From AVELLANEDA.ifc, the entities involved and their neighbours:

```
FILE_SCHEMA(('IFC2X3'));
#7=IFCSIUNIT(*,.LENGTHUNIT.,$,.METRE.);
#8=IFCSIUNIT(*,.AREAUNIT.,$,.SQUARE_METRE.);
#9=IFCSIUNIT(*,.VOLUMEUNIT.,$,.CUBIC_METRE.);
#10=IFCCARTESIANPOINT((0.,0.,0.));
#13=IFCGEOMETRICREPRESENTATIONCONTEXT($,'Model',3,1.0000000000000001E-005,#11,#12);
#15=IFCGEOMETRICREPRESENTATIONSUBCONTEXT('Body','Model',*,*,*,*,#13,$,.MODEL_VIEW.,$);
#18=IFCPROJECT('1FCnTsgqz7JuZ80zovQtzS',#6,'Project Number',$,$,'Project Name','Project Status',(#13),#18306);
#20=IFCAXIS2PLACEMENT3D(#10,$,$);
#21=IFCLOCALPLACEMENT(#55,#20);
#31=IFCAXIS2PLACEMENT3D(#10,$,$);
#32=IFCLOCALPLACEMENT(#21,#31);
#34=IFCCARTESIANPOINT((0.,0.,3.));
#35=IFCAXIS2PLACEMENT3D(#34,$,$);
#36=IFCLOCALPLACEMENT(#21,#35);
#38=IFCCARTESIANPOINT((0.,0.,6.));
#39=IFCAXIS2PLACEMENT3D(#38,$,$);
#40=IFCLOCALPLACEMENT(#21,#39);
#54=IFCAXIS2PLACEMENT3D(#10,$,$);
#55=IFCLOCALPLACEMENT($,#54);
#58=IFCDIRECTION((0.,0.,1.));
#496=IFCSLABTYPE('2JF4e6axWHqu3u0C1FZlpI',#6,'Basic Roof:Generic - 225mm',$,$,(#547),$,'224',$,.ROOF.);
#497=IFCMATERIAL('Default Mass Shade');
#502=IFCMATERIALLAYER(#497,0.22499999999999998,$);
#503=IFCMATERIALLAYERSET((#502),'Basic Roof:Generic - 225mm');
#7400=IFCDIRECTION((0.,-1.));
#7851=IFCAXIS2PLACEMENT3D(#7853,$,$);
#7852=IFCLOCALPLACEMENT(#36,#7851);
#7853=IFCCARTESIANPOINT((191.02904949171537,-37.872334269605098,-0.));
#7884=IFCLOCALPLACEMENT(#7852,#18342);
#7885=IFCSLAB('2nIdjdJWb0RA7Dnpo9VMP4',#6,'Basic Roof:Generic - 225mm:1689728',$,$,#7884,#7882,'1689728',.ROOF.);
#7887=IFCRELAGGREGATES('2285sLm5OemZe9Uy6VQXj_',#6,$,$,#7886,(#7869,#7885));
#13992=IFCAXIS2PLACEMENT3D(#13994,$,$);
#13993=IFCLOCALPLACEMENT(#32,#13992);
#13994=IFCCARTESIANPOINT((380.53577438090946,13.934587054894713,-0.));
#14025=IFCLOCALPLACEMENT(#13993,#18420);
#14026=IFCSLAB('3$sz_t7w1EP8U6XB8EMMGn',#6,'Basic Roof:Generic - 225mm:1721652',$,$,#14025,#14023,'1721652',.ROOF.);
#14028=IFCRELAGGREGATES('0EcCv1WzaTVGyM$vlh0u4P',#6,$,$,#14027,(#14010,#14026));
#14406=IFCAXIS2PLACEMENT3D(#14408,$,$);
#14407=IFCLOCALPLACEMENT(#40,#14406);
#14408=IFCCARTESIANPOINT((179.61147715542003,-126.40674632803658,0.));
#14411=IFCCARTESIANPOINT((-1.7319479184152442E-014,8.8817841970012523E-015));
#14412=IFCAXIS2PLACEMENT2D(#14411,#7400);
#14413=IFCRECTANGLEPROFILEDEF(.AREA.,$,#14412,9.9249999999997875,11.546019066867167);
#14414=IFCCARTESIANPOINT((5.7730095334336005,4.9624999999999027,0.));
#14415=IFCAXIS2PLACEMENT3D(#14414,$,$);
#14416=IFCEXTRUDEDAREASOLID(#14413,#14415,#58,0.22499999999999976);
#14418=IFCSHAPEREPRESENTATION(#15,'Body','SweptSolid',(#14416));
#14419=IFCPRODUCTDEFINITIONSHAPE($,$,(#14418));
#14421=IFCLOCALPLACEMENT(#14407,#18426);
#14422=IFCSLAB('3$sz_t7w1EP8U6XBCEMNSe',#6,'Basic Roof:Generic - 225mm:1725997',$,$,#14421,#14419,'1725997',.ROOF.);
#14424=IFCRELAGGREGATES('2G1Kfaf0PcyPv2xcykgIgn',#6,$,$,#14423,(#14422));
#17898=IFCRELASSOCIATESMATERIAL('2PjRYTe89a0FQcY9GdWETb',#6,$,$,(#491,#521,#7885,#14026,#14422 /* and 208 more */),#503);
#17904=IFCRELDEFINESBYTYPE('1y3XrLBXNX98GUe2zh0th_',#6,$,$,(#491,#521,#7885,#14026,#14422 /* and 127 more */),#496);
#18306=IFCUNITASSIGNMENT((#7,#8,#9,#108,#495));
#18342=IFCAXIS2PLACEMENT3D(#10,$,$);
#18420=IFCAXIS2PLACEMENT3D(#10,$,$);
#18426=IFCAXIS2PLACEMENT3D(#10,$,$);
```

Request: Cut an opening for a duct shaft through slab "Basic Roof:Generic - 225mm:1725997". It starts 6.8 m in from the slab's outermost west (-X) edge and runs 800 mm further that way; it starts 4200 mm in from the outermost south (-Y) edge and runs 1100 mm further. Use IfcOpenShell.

```python
import numpy as np
import ifcopenshell
import ifcopenshell.api.feature
import ifcopenshell.api.geometry
import ifcopenshell.api.root
import ifcopenshell.geom
import ifcopenshell.util.placement
import ifcopenshell.util.representation
import ifcopenshell.util.shape
import ifcopenshell.util.unit

model = ifcopenshell.open("AVELLANEDA.ifc")
unit_scale = ifcopenshell.util.unit.calculate_unit_scale(model)
settings = ifcopenshell.geom.settings()


def volume(element):
    """Net volume in cubic metres, openings subtracted."""
    shape = ifcopenshell.geom.create_shape(settings, element)
    return ifcopenshell.util.shape.get_volume(shape.geometry)


slab = model.by_guid("3$sz_t7w1EP8U6XBCEMNSe")
before = volume(slab)

# Extent in the slab's own axes, in metres. The edges named are its -X and -Y sides.
slab_shape = ifcopenshell.geom.create_shape(settings, slab)
vertices = ifcopenshell.util.shape.get_vertices(slab_shape.geometry)
x_min, y_min, bottom = vertices.min(axis=0)
top = vertices[:, 2].max()

opening = ifcopenshell.api.root.create_entity(model, ifc_class="IfcOpeningElement", name="Duct shaft opening")
context = ifcopenshell.util.representation.get_context(model, "Model", "Body", "MODEL_VIEW")
width, depth = 0.8, 1.1
outline = [(0.0, 0.0), (width, 0.0), (width, depth), (0.0, depth), (0.0, 0.0)]
# Overshoot both faces by 50 mm so the cut is clean.
shape = ifcopenshell.api.geometry.add_slab_representation(
    model, context=context, depth=top - bottom + 0.1, polyline=outline
)
ifcopenshell.api.geometry.assign_representation(model, product=opening, representation=shape)

matrix = ifcopenshell.util.placement.get_local_placement(slab.ObjectPlacement)
matrix[:, 3] = matrix @ np.append(np.array([x_min + 6.8, y_min + 4.2, bottom - 0.05]) / unit_scale, 1.0)
ifcopenshell.api.geometry.edit_object_placement(model, product=opening, matrix=matrix, is_si=False)
ifcopenshell.api.feature.add_feature(model, feature=opening, element=slab)

after = volume(slab)

print(f"slab volume {before:.3f} -> {after:.3f} m3")

model.write("AVELLANEDA_v2.ifc")
```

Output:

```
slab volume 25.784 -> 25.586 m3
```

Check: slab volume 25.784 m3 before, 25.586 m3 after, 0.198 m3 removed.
